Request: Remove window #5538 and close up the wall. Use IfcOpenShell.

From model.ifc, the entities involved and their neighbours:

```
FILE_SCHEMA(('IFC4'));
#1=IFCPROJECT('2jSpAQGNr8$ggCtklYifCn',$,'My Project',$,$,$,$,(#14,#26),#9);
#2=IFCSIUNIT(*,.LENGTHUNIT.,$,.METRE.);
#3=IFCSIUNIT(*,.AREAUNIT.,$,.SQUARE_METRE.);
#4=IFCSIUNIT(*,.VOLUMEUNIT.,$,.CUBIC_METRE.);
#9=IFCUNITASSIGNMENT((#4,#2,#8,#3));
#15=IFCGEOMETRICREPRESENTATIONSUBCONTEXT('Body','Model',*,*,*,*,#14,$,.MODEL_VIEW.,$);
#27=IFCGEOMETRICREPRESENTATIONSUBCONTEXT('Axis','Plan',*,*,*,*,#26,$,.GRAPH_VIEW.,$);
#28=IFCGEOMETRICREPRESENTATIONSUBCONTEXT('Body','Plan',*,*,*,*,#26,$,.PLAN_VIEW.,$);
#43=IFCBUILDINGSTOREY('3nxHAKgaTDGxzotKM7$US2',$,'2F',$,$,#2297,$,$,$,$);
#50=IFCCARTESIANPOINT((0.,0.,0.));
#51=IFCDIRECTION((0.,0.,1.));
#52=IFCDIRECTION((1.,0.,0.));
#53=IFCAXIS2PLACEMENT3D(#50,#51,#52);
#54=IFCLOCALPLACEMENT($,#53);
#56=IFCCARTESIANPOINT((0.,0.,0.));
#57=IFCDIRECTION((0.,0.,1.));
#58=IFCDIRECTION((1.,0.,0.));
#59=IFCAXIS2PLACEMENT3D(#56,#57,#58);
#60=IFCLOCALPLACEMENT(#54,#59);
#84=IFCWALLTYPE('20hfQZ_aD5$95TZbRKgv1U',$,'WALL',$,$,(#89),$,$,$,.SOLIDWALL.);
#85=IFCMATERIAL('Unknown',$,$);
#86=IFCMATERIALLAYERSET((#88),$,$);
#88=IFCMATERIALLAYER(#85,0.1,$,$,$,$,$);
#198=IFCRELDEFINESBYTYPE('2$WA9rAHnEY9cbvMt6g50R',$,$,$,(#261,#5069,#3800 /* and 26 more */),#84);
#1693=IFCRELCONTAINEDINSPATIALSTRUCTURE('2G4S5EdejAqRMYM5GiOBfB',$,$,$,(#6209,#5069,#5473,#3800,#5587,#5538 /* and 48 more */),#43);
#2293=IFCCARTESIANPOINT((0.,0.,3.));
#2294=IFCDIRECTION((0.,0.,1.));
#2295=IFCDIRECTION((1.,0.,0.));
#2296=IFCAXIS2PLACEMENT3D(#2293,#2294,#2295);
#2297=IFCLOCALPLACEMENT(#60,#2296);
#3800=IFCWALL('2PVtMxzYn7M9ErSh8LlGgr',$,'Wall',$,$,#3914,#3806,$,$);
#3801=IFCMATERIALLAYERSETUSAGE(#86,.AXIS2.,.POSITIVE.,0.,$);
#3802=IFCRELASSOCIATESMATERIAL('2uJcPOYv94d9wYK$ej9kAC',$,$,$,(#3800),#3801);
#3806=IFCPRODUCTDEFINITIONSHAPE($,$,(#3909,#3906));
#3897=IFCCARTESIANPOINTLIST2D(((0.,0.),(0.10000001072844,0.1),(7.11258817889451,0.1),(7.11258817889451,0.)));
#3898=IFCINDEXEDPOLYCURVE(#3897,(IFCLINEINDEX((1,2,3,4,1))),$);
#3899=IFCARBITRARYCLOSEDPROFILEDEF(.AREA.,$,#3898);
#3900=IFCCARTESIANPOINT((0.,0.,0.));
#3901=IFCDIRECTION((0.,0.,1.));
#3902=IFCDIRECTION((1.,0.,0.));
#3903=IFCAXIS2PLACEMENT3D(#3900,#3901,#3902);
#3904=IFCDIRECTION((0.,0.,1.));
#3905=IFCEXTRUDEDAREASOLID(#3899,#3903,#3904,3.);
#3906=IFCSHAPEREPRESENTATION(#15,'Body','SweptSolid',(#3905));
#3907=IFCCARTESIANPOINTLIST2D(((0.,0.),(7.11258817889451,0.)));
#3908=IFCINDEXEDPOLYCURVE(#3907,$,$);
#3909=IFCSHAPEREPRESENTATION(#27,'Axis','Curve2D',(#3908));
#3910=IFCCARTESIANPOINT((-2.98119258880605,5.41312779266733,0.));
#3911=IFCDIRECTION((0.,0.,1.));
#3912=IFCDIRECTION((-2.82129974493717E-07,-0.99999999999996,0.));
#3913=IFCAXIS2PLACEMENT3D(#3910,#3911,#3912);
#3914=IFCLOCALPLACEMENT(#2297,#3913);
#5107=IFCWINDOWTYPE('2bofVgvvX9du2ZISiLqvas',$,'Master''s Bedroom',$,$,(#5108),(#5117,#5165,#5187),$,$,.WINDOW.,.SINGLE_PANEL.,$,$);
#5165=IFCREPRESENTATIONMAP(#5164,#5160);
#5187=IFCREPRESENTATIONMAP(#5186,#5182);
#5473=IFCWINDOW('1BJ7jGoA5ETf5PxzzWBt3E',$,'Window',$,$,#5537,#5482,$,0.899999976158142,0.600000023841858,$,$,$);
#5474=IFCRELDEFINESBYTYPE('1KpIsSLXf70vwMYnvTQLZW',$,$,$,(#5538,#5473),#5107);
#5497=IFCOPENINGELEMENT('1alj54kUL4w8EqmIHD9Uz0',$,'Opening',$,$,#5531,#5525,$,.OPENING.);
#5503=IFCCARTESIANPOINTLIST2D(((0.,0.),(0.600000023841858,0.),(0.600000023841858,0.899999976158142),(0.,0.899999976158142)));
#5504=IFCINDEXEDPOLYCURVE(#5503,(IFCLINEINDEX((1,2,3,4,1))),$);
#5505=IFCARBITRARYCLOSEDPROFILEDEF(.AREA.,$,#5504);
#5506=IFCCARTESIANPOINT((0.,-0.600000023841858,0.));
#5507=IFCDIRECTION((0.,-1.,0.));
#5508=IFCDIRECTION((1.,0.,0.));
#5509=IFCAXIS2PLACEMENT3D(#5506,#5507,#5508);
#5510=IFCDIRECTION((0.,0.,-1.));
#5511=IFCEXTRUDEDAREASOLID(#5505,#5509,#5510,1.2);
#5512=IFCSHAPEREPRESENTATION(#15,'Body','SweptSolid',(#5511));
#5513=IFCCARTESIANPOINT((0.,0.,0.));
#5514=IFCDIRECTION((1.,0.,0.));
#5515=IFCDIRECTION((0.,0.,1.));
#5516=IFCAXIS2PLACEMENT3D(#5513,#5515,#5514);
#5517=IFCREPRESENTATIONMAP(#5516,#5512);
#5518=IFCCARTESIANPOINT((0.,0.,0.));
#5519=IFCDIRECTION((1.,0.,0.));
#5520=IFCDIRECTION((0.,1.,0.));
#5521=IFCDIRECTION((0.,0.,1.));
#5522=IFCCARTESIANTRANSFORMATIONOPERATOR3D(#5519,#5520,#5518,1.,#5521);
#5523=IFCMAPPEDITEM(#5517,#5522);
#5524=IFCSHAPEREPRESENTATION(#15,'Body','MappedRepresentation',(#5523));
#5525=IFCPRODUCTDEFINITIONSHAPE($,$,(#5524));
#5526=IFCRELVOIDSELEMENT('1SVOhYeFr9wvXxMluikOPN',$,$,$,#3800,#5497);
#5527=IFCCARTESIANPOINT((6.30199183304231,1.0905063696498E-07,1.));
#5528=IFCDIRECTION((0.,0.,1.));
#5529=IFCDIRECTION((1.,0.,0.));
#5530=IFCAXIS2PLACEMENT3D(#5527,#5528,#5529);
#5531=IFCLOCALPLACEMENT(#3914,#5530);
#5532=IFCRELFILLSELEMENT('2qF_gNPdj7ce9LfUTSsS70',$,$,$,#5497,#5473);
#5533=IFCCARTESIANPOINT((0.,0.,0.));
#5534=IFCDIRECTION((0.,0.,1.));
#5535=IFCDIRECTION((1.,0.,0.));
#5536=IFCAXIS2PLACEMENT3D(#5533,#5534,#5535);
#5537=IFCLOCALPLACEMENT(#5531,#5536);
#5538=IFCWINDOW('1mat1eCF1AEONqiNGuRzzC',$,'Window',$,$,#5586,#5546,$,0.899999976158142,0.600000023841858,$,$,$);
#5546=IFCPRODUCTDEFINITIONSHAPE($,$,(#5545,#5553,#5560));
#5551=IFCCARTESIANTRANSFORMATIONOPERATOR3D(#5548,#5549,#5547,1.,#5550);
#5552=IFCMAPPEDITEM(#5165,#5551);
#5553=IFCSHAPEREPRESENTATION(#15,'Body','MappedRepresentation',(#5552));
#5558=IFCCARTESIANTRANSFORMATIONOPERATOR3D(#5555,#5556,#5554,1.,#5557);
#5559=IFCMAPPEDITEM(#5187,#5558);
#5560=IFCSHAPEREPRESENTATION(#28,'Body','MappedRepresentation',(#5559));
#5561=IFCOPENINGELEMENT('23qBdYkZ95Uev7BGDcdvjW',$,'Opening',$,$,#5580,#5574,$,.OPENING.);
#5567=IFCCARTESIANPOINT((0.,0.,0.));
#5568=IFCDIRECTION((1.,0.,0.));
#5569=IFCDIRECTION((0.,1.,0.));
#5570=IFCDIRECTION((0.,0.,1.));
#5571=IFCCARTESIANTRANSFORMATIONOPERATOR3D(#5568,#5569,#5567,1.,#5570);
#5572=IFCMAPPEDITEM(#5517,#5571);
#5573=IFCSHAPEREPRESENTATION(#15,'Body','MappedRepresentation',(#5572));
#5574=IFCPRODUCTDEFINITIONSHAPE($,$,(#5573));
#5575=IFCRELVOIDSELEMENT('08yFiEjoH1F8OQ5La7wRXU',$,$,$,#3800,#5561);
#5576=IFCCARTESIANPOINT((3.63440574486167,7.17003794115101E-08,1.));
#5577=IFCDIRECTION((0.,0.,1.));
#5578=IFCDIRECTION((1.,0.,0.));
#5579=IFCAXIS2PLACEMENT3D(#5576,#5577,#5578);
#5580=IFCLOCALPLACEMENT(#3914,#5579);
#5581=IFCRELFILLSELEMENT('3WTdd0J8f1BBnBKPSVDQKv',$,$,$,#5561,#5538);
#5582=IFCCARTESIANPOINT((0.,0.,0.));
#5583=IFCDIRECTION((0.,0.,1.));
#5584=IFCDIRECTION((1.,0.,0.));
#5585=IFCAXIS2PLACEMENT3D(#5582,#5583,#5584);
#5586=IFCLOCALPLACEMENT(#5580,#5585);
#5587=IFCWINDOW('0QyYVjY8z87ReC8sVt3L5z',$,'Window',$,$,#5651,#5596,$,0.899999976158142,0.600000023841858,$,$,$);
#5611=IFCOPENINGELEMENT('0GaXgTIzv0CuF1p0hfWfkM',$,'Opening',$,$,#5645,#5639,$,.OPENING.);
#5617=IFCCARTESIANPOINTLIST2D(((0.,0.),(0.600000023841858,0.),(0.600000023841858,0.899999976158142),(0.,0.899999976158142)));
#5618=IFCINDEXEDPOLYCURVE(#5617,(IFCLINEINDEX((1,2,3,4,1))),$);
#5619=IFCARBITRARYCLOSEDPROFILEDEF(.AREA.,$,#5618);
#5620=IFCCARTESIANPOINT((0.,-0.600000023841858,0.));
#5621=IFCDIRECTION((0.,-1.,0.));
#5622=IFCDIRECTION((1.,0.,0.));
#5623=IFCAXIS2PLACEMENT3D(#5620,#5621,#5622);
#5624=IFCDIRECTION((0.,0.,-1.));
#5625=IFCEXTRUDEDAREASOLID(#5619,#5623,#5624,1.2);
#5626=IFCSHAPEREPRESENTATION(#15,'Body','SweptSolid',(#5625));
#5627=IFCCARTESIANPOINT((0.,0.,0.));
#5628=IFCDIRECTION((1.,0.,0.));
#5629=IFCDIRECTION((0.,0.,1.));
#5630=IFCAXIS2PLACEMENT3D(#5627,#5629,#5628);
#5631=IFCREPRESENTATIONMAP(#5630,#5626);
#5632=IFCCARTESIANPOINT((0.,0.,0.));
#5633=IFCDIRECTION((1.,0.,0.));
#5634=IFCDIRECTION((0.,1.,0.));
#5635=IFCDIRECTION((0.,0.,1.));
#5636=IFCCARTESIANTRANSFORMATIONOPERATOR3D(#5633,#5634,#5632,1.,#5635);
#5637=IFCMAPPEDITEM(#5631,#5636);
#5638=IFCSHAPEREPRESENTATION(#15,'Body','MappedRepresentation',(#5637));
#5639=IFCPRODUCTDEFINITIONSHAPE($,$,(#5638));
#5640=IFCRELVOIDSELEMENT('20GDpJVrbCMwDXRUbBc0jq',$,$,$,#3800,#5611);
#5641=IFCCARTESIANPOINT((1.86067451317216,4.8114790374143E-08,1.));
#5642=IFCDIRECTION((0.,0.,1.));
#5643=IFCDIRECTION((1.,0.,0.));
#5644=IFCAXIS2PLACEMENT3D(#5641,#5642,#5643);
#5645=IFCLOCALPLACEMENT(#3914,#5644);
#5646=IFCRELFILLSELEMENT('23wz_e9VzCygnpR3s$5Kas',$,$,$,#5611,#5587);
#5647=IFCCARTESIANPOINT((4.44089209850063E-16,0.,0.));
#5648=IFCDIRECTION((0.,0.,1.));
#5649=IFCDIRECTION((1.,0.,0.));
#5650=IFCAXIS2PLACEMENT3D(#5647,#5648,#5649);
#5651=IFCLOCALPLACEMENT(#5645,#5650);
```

```python
import ifcopenshell
import ifcopenshell.api.feature
import ifcopenshell.api.root
import ifcopenshell.geom
import ifcopenshell.util.shape

model = ifcopenshell.open("model.ifc")
settings = ifcopenshell.geom.settings()


def volume(element):
    """Net volume in cubic metres, openings subtracted."""
    shape = ifcopenshell.geom.create_shape(settings, element)
    return ifcopenshell.util.shape.get_volume(shape.geometry)


window = model.by_guid("1mat1eCF1AEONqiNGuRzzC")
opening = window.FillsVoids[0].RelatingOpeningElement
wall = opening.VoidsElements[0].RelatingBuildingElement
before = volume(wall)

ifcopenshell.api.root.remove_product(model, product=window)
ifcopenshell.api.feature.remove_feature(model, feature=opening)

after = volume(wall)

print(f"wall volume {before:.3f} -> {after:.3f} m3")

model.write("model-out.ifc")
```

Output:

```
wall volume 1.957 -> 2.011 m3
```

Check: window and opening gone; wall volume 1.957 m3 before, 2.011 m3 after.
